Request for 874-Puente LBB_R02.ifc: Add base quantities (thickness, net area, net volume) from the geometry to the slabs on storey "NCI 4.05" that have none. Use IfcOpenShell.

First a look at what the model holds.

```python
import ifcopenshell
import ifcopenshell.util.element
import ifcopenshell.util.unit

model = ifcopenshell.open("874-Puente LBB_R02.ifc")
print(model.schema)
for unit_type in ("LENGTHUNIT", "AREAUNIT", "VOLUMEUNIT"):
    print(unit_type, ifcopenshell.util.unit.calculate_unit_scale(model, unit_type))
storey = next(s for s in model.by_type("IfcBuildingStorey") if s.Name == "NCI 4.05")
slabs = [e for e in ifcopenshell.util.element.get_decomposition(storey) if e.is_a("IfcSlab")]
for e in sorted(slabs, key=lambda e: e.id()):
    print(e.id(), e.is_a(), e.Name, list(ifcopenshell.util.element.get_psets(e, qtos_only=True)), sep=" | ")
```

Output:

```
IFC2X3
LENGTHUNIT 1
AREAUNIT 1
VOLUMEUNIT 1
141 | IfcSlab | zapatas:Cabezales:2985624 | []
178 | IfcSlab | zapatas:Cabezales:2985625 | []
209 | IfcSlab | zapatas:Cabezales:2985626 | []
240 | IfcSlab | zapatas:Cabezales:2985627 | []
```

```python
import ifcopenshell
import ifcopenshell.api.pset
import ifcopenshell.geom
import ifcopenshell.util.element
import ifcopenshell.util.shape
import ifcopenshell.util.unit

model = ifcopenshell.open("874-Puente LBB_R02.ifc")
unit_scale = ifcopenshell.util.unit.calculate_unit_scale(model)
area_scale = ifcopenshell.util.unit.calculate_unit_scale(model, "AREAUNIT")
volume_scale = ifcopenshell.util.unit.calculate_unit_scale(model, "VOLUMEUNIT")
settings = ifcopenshell.geom.settings()

storey = next(s for s in model.by_type("IfcBuildingStorey") if s.Name == "NCI 4.05")
slabs = [e for e in ifcopenshell.util.element.get_decomposition(storey) if e.is_a("IfcSlab")]

for e in sorted(slabs, key=lambda e: e.id()):
    if ifcopenshell.util.element.get_psets(e, qtos_only=True, should_inherit=False):
        continue
    # Geometry comes back in metres, in the element's own axes.
    shape = ifcopenshell.geom.create_shape(settings, e)
    values = {
        "Width": ifcopenshell.util.shape.get_z(shape.geometry) / unit_scale,
        "NetArea": ifcopenshell.util.shape.get_footprint_area(shape.geometry) / area_scale,
        "NetVolume": ifcopenshell.util.shape.get_volume(shape.geometry) / volume_scale,
    }
    qto = ifcopenshell.api.pset.add_qto(model, product=e, name="BaseQuantities")
    ifcopenshell.api.pset.edit_qto(model, qto=qto, properties=values)
    print(e.id(), {k: round(v, 3) for k, v in values.items()})

model.write("874-Puente LBB_R02_updated.ifc")
```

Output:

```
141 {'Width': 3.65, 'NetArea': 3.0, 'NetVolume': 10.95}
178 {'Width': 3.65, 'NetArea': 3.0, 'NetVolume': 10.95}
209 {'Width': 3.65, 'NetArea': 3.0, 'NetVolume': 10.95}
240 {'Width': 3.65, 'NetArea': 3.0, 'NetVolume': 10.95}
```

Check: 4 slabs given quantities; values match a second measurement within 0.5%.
